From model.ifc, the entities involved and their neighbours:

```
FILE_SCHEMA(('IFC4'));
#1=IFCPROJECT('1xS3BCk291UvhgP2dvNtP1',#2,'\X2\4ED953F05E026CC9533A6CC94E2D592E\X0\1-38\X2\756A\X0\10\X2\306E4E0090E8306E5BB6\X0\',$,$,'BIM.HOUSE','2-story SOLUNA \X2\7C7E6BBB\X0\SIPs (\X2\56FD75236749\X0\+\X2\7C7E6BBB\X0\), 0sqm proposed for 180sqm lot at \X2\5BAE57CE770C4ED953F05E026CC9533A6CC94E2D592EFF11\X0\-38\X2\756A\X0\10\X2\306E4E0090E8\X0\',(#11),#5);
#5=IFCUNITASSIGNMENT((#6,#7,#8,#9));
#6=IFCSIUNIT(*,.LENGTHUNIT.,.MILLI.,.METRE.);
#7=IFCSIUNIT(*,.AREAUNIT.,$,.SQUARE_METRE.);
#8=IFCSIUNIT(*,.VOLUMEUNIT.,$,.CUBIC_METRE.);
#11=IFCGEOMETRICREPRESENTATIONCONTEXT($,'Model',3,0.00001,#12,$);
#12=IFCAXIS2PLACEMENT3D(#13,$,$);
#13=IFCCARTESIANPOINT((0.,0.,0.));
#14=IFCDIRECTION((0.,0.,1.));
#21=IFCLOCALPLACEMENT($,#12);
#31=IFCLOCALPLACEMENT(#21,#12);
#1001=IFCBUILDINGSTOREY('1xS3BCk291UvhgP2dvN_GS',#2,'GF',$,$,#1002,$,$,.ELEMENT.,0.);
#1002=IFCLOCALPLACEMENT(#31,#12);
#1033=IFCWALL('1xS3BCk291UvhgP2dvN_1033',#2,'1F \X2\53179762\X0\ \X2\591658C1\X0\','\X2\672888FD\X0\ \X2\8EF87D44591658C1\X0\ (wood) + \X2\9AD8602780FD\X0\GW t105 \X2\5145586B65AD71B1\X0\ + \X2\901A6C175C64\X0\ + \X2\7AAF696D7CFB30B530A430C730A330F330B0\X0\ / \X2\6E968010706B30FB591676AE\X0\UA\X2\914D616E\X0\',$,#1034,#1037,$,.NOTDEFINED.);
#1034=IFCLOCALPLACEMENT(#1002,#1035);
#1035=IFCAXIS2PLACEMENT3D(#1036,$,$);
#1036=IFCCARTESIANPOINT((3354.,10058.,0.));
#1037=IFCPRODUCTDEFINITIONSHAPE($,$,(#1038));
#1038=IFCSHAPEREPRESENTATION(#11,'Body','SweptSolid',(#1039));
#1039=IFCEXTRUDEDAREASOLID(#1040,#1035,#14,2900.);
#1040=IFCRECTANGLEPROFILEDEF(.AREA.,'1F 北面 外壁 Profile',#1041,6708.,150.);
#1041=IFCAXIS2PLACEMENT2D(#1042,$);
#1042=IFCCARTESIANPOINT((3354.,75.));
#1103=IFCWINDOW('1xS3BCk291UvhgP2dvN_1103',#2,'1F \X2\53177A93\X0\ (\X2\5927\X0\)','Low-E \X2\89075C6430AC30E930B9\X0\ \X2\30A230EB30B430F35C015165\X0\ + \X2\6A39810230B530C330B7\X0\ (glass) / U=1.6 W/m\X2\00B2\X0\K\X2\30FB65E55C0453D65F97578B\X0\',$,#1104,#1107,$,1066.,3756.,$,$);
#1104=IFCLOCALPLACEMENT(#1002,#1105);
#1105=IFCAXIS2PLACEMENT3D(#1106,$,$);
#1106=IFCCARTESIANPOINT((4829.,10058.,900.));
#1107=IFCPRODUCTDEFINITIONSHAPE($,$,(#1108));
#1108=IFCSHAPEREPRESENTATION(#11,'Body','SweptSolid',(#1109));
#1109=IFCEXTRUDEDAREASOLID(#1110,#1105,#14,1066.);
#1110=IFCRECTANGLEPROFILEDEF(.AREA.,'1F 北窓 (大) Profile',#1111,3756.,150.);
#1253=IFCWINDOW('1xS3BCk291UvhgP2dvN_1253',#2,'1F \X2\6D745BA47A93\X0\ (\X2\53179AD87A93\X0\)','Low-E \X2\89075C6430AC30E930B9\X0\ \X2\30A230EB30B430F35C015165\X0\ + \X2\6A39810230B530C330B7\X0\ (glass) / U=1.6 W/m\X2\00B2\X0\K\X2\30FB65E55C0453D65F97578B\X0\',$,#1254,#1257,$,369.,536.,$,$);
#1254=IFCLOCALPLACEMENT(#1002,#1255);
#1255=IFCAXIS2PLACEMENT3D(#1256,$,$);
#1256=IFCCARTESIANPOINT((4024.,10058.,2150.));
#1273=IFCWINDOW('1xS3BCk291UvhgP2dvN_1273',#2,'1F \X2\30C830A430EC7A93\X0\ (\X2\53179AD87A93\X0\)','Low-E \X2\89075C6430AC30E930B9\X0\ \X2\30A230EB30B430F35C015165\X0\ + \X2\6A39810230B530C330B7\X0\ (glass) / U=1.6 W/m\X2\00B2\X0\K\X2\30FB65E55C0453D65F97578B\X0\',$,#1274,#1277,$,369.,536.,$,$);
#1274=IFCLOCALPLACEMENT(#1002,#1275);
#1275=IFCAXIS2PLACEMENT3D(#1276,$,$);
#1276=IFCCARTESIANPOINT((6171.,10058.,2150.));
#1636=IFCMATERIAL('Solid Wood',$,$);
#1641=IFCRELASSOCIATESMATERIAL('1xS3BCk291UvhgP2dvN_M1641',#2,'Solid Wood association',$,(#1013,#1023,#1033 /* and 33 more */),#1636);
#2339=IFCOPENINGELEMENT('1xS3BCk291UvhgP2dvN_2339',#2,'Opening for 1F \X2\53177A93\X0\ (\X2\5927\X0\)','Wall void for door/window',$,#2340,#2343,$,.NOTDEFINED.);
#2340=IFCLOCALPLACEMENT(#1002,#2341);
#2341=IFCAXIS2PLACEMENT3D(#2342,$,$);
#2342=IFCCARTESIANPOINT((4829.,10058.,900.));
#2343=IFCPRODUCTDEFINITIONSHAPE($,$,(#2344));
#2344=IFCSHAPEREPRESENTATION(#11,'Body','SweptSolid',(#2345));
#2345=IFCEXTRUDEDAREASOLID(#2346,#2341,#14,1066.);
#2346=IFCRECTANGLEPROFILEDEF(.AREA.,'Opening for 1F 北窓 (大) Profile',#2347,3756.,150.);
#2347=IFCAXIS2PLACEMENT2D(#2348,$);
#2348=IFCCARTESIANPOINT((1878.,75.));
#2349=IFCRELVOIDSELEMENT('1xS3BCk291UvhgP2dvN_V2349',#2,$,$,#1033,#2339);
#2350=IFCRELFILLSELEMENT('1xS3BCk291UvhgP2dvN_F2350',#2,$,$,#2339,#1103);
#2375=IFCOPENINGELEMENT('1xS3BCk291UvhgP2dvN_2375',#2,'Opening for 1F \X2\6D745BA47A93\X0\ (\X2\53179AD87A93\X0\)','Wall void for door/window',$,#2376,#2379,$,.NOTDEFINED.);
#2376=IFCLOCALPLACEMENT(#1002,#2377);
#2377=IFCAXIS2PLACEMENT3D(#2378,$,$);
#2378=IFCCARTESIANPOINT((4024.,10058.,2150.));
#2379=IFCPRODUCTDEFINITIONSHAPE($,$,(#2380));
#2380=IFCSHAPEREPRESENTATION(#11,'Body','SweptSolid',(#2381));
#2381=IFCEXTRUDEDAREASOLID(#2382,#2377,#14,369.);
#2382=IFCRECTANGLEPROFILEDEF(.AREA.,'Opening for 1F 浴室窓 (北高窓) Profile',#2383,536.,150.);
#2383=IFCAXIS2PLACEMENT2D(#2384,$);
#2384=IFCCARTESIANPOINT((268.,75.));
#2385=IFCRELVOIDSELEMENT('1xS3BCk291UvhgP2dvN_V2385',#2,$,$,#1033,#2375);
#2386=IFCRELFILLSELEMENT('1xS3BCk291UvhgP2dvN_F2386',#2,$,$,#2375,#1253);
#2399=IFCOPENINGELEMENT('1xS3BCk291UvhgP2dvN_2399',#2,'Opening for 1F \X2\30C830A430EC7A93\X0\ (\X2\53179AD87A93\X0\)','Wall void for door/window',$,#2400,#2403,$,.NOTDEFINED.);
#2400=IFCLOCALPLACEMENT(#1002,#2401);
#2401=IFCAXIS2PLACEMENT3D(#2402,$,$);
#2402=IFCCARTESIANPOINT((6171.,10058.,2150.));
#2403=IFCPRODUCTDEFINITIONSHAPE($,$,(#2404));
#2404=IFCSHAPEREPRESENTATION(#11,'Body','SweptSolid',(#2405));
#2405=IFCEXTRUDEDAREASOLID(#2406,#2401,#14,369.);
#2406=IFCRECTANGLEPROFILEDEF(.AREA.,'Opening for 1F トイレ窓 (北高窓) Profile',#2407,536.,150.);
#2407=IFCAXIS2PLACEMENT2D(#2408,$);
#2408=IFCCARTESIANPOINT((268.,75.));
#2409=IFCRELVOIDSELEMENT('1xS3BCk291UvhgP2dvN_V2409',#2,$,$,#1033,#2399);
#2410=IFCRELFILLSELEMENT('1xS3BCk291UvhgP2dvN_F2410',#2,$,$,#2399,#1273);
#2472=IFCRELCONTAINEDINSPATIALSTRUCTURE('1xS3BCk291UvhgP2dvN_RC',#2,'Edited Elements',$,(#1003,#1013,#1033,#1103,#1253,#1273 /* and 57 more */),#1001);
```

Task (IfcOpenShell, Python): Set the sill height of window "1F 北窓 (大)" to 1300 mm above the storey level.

```python
import numpy as np
import ifcopenshell
import ifcopenshell.api.geometry
import ifcopenshell.geom
import ifcopenshell.util.element
import ifcopenshell.util.placement
import ifcopenshell.util.shape
import ifcopenshell.util.unit

model = ifcopenshell.open("model.ifc")
unit_scale = ifcopenshell.util.unit.calculate_unit_scale(model)

window = model.by_guid("1xS3BCk291UvhgP2dvN_1103")
opening = window.FillsVoids[0].RelatingOpeningElement
storey = ifcopenshell.util.element.get_container(window, ifc_class="IfcBuildingStorey")
level = ifcopenshell.util.placement.get_local_placement(storey.ObjectPlacement)[2, 3]

# The opening's origin need not be at the sill, so measure its lowest point.
shape = ifcopenshell.geom.create_shape(ifcopenshell.geom.settings(), opening)
bottom = ifcopenshell.util.shape.get_shape_bottom_elevation(shape, shape.geometry) / unit_scale
dz = level + 1.3 / unit_scale - bottom

shift = np.array([0.0, 0.0, dz])
# The window is not placed relative to its opening, so move both.
for product in (opening, window):
    matrix = ifcopenshell.util.placement.get_local_placement(product.ObjectPlacement)
    matrix[:3, 3] += shift
    ifcopenshell.api.geometry.edit_object_placement(model, product=product, matrix=matrix, is_si=False)

print(f"moved by {dz * unit_scale:+.3f} m")

model.write("model_rev.ifc")
```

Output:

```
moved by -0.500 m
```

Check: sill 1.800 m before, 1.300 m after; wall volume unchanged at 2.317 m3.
